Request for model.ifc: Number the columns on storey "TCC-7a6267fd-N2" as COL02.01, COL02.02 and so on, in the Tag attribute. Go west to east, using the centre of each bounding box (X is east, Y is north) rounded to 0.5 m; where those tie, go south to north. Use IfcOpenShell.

First a look at what the model holds.

```python
import ifcopenshell
import ifcopenshell.util.element
import ifcopenshell.util.placement

model = ifcopenshell.open("model.ifc")
print(model.schema)
storey = next(s for s in model.by_type("IfcBuildingStorey") if s.Name == "TCC-7a6267fd-N2")
columns = [e for e in ifcopenshell.util.element.get_decomposition(storey) if e.is_a("IfcColumn")]
for e in sorted(columns, key=lambda e: e.id()):
    origin = ifcopenshell.util.placement.get_local_placement(e.ObjectPlacement)[:3, 3]
    print(e.id(), e.Tag, e.Name, origin.round(2) + 0.0, sep=" | ")
```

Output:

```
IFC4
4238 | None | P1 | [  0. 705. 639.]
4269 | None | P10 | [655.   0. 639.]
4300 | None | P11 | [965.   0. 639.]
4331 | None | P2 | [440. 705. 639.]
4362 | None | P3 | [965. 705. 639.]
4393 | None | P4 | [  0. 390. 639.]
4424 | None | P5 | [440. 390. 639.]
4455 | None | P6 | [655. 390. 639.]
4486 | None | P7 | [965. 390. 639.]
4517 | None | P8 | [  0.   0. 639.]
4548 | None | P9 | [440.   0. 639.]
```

```python
import ifcopenshell
import ifcopenshell.geom
import ifcopenshell.util.element
import ifcopenshell.util.shape

model = ifcopenshell.open("model.ifc")
settings = ifcopenshell.geom.settings()
settings.set("use-world-coords", True)


def centre(element):
    shape = ifcopenshell.geom.create_shape(settings, element)
    return ifcopenshell.util.shape.get_bbox_centroid(shape.geometry)


storey = next(s for s in model.by_type("IfcBuildingStorey") if s.Name == "TCC-7a6267fd-N2")
columns = [e for e in ifcopenshell.util.element.get_decomposition(storey) if e.is_a("IfcColumn")]

# Insertion points can sit at a corner or the storey origin, so sort by the geometry (in metres).
centres = {e: centre(e) for e in columns}
columns.sort(key=lambda e: (round(centres[e][0] / 0.5), centres[e][1]))

for i, e in enumerate(columns, start=1):
    number = f"COL02.{i:02d}"
    e.Tag = number
    print(e.id(), number)

model.write("model_v2.ifc")
```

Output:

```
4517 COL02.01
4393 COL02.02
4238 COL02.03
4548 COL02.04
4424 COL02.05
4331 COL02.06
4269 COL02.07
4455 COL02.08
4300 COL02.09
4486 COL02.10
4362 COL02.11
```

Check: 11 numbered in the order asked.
